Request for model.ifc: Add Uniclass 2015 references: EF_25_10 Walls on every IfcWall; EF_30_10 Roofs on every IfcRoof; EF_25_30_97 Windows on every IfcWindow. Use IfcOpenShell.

First a look at what the model holds.

```python
import ifcopenshell

model = ifcopenshell.open("model.ifc")
print(model.schema)
print("classifications:", [c.Name for c in model.by_type("IfcClassification")])
for ifc_class in ("IfcDoor", "IfcRoof", "IfcStair", "IfcWall", "IfcWindow"):
    print(ifc_class, len(model.by_type(ifc_class)))
```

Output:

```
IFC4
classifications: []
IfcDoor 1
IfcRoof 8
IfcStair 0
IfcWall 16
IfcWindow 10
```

```python
import ifcopenshell
import ifcopenshell.api.classification

model = ifcopenshell.open("model.ifc")

system = ifcopenshell.api.classification.add_classification(model, classification="Uniclass 2015")

codes = {
    "IfcWall": ("EF_25_10", "Walls"),
    "IfcRoof": ("EF_30_10", "Roofs"),
    "IfcWindow": ("EF_25_30_97", "Windows"),
}
for ifc_class, (code, name) in codes.items():
    products = model.by_type(ifc_class)
    ifcopenshell.api.classification.add_reference(
        model, products=products, classification=system, identification=code, name=name
    )
    print(code, len(products))

model.write("model_rev.ifc")
```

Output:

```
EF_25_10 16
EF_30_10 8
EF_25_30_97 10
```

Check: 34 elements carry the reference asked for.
